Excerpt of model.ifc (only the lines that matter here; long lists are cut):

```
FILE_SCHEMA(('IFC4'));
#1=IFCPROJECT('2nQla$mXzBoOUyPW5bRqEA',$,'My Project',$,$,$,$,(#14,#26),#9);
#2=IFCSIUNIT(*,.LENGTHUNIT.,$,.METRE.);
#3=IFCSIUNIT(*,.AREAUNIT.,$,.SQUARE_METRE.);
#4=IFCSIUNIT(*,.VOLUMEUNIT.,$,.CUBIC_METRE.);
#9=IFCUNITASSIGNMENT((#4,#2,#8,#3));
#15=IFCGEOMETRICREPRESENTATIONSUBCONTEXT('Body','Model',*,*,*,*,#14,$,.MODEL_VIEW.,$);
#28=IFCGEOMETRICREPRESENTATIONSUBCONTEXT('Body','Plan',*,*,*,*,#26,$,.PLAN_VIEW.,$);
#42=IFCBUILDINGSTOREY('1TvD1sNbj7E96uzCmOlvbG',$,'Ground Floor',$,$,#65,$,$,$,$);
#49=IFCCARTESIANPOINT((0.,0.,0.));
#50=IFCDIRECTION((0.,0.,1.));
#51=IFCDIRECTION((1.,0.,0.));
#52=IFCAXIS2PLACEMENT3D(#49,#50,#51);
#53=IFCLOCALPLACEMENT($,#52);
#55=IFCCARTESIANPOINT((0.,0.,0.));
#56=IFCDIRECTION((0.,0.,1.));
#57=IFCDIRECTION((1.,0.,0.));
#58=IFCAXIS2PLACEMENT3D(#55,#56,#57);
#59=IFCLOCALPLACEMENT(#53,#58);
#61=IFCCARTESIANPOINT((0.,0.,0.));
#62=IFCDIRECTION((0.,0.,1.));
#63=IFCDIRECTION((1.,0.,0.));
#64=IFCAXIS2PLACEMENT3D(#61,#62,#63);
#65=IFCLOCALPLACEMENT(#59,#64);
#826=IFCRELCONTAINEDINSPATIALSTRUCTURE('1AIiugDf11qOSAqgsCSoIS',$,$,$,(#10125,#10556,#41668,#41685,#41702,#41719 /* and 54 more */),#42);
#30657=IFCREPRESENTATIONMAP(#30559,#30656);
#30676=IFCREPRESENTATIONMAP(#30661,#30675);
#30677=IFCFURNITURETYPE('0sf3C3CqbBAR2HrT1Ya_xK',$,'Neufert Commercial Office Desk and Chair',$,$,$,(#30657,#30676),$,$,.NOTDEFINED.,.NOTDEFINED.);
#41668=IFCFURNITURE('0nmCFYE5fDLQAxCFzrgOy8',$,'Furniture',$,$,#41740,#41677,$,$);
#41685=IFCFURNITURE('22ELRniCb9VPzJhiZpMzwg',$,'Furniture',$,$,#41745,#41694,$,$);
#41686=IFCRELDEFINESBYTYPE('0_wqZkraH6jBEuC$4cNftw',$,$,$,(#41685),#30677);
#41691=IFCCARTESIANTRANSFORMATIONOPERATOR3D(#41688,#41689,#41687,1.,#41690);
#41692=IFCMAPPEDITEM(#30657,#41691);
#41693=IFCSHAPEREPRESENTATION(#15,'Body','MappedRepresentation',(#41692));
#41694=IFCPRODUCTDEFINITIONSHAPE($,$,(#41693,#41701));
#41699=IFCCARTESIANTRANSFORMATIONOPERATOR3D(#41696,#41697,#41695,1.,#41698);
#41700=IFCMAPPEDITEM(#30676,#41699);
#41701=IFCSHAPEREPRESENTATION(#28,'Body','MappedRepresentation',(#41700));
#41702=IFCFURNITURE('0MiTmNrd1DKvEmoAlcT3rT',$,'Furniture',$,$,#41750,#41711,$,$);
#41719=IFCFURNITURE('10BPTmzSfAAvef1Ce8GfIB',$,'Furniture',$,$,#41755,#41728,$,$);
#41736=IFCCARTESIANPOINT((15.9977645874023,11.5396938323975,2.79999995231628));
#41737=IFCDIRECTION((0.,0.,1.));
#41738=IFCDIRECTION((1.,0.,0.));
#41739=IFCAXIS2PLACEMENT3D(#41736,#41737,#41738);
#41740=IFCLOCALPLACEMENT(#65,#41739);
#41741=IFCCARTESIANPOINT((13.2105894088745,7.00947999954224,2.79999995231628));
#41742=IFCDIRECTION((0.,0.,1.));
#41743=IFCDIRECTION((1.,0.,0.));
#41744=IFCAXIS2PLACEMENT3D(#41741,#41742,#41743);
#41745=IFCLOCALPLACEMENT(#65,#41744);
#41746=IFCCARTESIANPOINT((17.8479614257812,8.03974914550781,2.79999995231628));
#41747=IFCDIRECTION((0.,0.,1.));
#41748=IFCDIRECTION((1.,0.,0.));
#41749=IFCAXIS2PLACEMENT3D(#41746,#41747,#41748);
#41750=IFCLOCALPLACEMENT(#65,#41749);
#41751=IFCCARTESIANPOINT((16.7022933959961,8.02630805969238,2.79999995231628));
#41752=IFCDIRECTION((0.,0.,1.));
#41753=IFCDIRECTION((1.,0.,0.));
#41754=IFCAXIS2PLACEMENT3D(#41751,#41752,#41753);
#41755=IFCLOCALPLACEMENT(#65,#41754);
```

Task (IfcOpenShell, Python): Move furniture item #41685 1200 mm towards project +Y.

```python
import ifcopenshell
import ifcopenshell.api.geometry
import ifcopenshell.util.placement
import ifcopenshell.util.unit

model = ifcopenshell.open("model.ifc")
unit_scale = ifcopenshell.util.unit.calculate_unit_scale(model)

item = model.by_guid("22ELRniCb9VPzJhiZpMzwg")
matrix = ifcopenshell.util.placement.get_local_placement(item.ObjectPlacement)
matrix[1, 3] += 1.2 / unit_scale
ifcopenshell.api.geometry.edit_object_placement(model, product=item, matrix=matrix, is_si=False)

print(ifcopenshell.util.placement.get_local_placement(item.ObjectPlacement).round(3) + 0.0)

model.write("model-out.ifc")
```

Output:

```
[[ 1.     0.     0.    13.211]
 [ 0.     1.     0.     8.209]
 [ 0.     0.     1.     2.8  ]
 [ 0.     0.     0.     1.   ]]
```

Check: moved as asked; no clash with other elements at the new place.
